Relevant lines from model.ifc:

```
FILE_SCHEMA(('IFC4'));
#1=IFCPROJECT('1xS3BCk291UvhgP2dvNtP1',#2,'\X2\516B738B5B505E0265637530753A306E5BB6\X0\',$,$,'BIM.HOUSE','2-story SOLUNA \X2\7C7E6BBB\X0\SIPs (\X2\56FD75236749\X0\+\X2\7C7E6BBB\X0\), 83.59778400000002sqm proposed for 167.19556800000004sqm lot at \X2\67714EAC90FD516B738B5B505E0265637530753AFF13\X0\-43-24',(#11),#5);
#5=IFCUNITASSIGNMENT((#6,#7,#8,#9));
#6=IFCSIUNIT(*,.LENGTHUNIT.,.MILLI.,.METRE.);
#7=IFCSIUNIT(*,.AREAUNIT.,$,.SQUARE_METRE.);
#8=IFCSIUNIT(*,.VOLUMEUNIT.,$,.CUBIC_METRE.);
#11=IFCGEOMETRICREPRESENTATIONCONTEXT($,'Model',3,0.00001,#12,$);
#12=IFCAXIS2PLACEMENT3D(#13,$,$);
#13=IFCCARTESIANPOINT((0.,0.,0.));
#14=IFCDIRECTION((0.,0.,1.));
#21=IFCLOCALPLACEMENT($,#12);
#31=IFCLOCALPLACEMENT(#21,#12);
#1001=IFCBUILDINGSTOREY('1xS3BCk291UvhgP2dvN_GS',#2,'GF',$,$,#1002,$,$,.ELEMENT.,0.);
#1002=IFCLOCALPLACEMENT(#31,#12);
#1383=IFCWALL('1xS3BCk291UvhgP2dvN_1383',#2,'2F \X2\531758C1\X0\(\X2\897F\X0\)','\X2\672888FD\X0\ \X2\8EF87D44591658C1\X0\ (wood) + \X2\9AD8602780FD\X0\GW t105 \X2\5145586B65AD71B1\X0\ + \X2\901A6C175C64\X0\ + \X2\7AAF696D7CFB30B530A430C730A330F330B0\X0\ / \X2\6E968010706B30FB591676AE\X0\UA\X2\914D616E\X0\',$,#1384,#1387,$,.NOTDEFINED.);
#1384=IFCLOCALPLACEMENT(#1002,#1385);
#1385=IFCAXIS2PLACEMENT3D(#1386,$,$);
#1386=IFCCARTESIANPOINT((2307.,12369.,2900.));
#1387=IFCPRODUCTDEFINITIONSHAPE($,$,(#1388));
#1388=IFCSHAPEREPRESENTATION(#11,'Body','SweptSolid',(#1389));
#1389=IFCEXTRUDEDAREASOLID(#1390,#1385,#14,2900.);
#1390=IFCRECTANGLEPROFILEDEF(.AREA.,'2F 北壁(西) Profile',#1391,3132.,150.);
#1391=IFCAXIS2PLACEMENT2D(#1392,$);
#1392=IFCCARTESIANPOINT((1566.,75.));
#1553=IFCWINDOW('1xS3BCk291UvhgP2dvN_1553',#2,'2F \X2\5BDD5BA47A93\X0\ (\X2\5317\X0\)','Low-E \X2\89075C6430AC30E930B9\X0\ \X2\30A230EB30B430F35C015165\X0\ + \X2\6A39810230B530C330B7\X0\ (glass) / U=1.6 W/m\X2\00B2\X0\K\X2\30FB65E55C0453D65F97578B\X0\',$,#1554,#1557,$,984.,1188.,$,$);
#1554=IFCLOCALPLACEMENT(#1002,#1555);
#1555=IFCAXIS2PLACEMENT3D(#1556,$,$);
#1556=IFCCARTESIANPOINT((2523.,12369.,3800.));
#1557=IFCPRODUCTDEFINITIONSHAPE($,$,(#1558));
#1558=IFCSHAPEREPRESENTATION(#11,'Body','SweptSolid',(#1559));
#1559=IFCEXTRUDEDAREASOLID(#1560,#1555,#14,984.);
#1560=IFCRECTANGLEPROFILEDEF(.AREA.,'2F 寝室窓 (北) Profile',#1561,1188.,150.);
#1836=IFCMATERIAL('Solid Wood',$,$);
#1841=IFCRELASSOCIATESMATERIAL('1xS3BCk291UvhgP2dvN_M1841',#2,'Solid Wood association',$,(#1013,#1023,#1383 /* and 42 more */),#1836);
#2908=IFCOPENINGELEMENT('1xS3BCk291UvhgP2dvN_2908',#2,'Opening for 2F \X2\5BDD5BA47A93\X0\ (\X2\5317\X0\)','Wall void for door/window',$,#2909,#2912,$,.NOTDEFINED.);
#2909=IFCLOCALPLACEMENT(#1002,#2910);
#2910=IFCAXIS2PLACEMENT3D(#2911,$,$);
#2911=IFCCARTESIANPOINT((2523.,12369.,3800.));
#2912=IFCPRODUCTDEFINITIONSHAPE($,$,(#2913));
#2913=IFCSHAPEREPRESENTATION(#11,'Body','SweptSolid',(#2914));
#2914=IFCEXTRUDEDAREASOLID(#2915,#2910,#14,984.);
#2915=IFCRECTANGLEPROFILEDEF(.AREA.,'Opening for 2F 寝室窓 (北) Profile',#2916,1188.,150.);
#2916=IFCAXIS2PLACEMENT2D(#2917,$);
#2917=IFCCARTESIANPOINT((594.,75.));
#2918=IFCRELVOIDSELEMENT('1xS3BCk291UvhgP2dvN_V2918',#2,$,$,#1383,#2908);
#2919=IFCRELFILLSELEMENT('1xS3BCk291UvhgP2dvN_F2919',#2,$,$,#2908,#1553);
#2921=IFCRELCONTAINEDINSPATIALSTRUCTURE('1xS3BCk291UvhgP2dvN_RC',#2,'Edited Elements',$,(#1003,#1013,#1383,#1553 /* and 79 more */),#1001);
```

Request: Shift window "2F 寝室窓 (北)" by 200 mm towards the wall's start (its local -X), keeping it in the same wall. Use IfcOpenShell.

```python
import ifcopenshell
import ifcopenshell.api.geometry
import ifcopenshell.util.placement
import ifcopenshell.util.unit

model = ifcopenshell.open("model.ifc")
unit_scale = ifcopenshell.util.unit.calculate_unit_scale(model)

window = model.by_guid("1xS3BCk291UvhgP2dvN_1553")
opening = window.FillsVoids[0].RelatingOpeningElement
wall = opening.VoidsElements[0].RelatingBuildingElement

wall_matrix = ifcopenshell.util.placement.get_local_placement(wall.ObjectPlacement)
shift = wall_matrix[:3, 0] * -0.2 / unit_scale
before = ifcopenshell.util.placement.get_local_placement(window.ObjectPlacement)[:3, 3].copy()

# The window is not placed relative to its opening, so move both.
for product in (opening, window):
    matrix = ifcopenshell.util.placement.get_local_placement(product.ObjectPlacement)
    matrix[:3, 3] += shift
    ifcopenshell.api.geometry.edit_object_placement(model, product=product, matrix=matrix, is_si=False)

after = ifcopenshell.util.placement.get_local_placement(window.ObjectPlacement)[:3, 3]
print("window moved by", (after - before).round(3) + 0.0)

model.write("model_edited.ifc")
```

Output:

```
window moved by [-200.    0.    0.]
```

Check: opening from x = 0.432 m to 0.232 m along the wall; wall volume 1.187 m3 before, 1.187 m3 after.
